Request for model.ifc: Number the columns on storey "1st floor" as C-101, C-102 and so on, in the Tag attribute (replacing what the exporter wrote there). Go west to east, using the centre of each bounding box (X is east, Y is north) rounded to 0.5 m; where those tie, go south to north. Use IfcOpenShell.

First a look at what the model holds.

```python
import ifcopenshell
import ifcopenshell.util.element
import ifcopenshell.util.placement

model = ifcopenshell.open("model.ifc")
print(model.schema)
storey = next(s for s in model.by_type("IfcBuildingStorey") if s.Name == "1st floor")
columns = [e for e in ifcopenshell.util.element.get_decomposition(storey) if e.is_a("IfcColumn")]
for e in sorted(columns, key=lambda e: e.id()):
    origin = ifcopenshell.util.placement.get_local_placement(e.ObjectPlacement)[:3, 3]
    print(e.id(), e.Tag, e.Name, origin.round(2) + 0.0, sep=" | ")
```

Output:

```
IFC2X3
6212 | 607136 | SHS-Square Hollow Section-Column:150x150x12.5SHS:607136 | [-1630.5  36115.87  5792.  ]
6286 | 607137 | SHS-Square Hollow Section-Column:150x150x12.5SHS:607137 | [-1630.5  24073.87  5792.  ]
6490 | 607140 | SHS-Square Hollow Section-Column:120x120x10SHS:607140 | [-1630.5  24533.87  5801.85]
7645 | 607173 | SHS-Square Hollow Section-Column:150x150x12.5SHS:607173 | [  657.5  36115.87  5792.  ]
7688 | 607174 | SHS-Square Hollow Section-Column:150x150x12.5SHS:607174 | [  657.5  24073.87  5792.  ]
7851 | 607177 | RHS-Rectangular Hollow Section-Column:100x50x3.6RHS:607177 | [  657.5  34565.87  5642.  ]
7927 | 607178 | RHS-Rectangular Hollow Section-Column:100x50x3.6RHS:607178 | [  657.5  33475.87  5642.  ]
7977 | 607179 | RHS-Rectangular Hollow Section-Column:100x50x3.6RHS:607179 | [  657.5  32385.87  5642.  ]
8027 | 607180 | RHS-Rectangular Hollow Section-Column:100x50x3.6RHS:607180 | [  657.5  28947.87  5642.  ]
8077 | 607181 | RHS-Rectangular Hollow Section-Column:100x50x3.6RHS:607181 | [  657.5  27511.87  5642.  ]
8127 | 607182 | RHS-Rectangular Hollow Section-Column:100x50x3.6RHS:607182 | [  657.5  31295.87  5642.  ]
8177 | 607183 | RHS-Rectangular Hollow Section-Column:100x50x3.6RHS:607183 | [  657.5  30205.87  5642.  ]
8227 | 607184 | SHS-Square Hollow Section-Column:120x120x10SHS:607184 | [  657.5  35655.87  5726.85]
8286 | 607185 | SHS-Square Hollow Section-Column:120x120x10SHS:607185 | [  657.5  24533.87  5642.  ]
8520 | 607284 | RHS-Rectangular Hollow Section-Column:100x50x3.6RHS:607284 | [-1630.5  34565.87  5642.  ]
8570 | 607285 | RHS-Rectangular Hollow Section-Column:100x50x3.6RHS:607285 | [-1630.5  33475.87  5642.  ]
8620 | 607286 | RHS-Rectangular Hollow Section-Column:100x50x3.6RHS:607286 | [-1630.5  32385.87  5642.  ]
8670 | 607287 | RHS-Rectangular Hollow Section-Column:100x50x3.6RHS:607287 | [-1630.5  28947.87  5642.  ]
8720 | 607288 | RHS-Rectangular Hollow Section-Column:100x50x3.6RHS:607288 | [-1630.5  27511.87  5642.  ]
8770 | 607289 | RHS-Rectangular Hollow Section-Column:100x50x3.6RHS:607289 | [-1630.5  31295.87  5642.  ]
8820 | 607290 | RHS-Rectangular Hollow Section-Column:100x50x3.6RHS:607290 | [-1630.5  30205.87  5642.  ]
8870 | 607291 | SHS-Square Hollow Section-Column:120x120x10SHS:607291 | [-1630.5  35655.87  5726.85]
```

```python
import ifcopenshell
import ifcopenshell.geom
import ifcopenshell.util.element
import ifcopenshell.util.shape

model = ifcopenshell.open("model.ifc")
settings = ifcopenshell.geom.settings()
settings.set("use-world-coords", True)


def centre(element):
    shape = ifcopenshell.geom.create_shape(settings, element)
    return ifcopenshell.util.shape.get_bbox_centroid(shape.geometry)


storey = next(s for s in model.by_type("IfcBuildingStorey") if s.Name == "1st floor")
columns = [e for e in ifcopenshell.util.element.get_decomposition(storey) if e.is_a("IfcColumn")]

# Insertion points can sit at a corner or the storey origin, so sort by the geometry (in metres).
centres = {e: centre(e) for e in columns}
columns.sort(key=lambda e: (round(centres[e][0] / 0.5), centres[e][1]))

for i, e in enumerate(columns, start=1):
    number = f"C-1{i:02d}"
    e.Tag = number
    print(e.id(), number)

model.write("model_rev.ifc")
```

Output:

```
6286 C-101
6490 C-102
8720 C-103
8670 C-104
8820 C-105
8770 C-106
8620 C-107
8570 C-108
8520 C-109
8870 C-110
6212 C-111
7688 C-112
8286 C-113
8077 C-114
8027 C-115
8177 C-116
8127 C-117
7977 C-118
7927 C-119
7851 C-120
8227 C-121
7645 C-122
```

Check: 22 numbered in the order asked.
